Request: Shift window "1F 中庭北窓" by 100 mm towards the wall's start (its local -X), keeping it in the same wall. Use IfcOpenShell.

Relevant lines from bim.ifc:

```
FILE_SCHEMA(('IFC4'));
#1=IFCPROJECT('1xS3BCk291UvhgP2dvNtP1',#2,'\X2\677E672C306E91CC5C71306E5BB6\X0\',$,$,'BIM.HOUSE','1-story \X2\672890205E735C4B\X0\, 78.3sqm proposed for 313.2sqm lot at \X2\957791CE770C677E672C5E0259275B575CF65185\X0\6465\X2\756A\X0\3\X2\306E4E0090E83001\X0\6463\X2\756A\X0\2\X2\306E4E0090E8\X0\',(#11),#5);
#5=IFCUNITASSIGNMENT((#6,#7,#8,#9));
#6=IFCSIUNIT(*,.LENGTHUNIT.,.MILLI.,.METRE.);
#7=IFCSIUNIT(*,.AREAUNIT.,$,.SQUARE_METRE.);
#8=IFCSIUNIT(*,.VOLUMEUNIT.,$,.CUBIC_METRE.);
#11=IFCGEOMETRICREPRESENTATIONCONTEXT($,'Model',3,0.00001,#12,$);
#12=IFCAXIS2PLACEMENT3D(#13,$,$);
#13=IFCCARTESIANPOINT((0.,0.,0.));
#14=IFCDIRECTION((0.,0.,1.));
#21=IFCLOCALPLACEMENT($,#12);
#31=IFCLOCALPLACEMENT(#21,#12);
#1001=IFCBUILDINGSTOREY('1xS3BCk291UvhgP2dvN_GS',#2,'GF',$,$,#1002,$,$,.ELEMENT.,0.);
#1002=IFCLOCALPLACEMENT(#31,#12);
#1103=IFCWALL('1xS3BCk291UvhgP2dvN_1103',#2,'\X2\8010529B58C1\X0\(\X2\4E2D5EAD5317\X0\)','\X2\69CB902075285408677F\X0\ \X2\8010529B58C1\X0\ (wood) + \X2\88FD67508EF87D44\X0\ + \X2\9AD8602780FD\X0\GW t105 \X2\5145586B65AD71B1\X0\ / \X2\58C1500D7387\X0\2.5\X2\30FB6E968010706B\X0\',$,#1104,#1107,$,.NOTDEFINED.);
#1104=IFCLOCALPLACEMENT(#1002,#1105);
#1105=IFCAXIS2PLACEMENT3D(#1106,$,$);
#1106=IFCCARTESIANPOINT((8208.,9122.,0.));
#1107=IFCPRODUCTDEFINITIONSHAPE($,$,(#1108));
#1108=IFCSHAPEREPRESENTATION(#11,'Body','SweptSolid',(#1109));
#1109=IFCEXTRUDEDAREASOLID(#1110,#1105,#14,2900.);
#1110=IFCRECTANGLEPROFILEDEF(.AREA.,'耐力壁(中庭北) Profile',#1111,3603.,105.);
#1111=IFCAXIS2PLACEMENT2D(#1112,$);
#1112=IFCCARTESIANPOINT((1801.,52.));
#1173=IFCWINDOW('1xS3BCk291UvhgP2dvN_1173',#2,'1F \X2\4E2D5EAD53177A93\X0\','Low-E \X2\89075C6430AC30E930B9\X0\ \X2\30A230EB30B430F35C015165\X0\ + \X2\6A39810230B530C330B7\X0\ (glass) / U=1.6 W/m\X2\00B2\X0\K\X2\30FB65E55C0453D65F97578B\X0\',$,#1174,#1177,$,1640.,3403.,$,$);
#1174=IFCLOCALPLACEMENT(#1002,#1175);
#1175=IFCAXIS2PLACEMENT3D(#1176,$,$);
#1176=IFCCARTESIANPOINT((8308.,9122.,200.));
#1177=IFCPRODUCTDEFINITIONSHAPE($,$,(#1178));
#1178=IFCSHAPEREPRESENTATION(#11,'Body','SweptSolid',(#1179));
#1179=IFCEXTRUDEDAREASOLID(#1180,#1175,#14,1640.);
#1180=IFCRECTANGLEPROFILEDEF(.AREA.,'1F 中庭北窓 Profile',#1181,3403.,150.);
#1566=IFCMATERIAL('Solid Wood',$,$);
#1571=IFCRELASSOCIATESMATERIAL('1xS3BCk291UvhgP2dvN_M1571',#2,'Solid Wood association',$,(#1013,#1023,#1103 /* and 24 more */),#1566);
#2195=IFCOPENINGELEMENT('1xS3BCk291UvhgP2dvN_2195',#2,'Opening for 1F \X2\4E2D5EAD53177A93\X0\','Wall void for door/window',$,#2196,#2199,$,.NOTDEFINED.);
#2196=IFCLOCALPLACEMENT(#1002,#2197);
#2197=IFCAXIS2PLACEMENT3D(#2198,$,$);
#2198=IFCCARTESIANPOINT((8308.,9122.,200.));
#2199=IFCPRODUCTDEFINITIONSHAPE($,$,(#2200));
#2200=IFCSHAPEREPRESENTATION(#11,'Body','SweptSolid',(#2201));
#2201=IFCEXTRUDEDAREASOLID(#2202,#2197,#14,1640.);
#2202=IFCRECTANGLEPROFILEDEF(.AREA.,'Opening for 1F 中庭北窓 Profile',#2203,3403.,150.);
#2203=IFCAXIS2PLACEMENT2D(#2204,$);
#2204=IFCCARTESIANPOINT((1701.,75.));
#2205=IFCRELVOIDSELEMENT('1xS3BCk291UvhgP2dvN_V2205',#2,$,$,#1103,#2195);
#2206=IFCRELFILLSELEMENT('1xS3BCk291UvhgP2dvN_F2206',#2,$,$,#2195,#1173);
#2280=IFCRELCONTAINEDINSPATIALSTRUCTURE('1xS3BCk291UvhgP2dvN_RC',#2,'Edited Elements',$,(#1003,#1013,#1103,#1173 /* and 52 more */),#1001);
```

```python
import ifcopenshell
import ifcopenshell.api.geometry
import ifcopenshell.util.placement
import ifcopenshell.util.unit

model = ifcopenshell.open("bim.ifc")
unit_scale = ifcopenshell.util.unit.calculate_unit_scale(model)

window = model.by_guid("1xS3BCk291UvhgP2dvN_1173")
opening = window.FillsVoids[0].RelatingOpeningElement
wall = opening.VoidsElements[0].RelatingBuildingElement

wall_matrix = ifcopenshell.util.placement.get_local_placement(wall.ObjectPlacement)
shift = wall_matrix[:3, 0] * -0.1 / unit_scale
before = ifcopenshell.util.placement.get_local_placement(window.ObjectPlacement)[:3, 3].copy()

# The window is not placed relative to its opening, so move both.
for product in (opening, window):
    matrix = ifcopenshell.util.placement.get_local_placement(product.ObjectPlacement)
    matrix[:3, 3] += shift
    ifcopenshell.api.geometry.edit_object_placement(model, product=product, matrix=matrix, is_si=False)

after = ifcopenshell.util.placement.get_local_placement(window.ObjectPlacement)[:3, 3]
print("window moved by", (after - before).round(3) + 0.0)

model.write("bim_rev.ifc")
```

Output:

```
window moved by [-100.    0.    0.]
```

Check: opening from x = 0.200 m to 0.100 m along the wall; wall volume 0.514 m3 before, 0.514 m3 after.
